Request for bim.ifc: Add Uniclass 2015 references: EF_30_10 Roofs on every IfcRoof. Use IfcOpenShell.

First a look at what the model holds.

```python
import ifcopenshell

model = ifcopenshell.open("bim.ifc")
print(model.schema)
print("classifications:", [c.Name for c in model.by_type("IfcClassification")])
for ifc_class in ("IfcDoor", "IfcRoof", "IfcStair", "IfcWall", "IfcWindow"):
    print(ifc_class, len(model.by_type(ifc_class)))
```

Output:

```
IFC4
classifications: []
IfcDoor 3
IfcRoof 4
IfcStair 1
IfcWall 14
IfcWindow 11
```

```python
import ifcopenshell
import ifcopenshell.api.classification

model = ifcopenshell.open("bim.ifc")

system = ifcopenshell.api.classification.add_classification(model, classification="Uniclass 2015")

codes = {
    "IfcRoof": ("EF_30_10", "Roofs"),
}
for ifc_class, (code, name) in codes.items():
    products = model.by_type(ifc_class)
    ifcopenshell.api.classification.add_reference(
        model, products=products, classification=system, identification=code, name=name
    )
    print(code, len(products))

model.write("bim_edited.ifc")
```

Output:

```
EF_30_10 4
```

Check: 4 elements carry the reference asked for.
